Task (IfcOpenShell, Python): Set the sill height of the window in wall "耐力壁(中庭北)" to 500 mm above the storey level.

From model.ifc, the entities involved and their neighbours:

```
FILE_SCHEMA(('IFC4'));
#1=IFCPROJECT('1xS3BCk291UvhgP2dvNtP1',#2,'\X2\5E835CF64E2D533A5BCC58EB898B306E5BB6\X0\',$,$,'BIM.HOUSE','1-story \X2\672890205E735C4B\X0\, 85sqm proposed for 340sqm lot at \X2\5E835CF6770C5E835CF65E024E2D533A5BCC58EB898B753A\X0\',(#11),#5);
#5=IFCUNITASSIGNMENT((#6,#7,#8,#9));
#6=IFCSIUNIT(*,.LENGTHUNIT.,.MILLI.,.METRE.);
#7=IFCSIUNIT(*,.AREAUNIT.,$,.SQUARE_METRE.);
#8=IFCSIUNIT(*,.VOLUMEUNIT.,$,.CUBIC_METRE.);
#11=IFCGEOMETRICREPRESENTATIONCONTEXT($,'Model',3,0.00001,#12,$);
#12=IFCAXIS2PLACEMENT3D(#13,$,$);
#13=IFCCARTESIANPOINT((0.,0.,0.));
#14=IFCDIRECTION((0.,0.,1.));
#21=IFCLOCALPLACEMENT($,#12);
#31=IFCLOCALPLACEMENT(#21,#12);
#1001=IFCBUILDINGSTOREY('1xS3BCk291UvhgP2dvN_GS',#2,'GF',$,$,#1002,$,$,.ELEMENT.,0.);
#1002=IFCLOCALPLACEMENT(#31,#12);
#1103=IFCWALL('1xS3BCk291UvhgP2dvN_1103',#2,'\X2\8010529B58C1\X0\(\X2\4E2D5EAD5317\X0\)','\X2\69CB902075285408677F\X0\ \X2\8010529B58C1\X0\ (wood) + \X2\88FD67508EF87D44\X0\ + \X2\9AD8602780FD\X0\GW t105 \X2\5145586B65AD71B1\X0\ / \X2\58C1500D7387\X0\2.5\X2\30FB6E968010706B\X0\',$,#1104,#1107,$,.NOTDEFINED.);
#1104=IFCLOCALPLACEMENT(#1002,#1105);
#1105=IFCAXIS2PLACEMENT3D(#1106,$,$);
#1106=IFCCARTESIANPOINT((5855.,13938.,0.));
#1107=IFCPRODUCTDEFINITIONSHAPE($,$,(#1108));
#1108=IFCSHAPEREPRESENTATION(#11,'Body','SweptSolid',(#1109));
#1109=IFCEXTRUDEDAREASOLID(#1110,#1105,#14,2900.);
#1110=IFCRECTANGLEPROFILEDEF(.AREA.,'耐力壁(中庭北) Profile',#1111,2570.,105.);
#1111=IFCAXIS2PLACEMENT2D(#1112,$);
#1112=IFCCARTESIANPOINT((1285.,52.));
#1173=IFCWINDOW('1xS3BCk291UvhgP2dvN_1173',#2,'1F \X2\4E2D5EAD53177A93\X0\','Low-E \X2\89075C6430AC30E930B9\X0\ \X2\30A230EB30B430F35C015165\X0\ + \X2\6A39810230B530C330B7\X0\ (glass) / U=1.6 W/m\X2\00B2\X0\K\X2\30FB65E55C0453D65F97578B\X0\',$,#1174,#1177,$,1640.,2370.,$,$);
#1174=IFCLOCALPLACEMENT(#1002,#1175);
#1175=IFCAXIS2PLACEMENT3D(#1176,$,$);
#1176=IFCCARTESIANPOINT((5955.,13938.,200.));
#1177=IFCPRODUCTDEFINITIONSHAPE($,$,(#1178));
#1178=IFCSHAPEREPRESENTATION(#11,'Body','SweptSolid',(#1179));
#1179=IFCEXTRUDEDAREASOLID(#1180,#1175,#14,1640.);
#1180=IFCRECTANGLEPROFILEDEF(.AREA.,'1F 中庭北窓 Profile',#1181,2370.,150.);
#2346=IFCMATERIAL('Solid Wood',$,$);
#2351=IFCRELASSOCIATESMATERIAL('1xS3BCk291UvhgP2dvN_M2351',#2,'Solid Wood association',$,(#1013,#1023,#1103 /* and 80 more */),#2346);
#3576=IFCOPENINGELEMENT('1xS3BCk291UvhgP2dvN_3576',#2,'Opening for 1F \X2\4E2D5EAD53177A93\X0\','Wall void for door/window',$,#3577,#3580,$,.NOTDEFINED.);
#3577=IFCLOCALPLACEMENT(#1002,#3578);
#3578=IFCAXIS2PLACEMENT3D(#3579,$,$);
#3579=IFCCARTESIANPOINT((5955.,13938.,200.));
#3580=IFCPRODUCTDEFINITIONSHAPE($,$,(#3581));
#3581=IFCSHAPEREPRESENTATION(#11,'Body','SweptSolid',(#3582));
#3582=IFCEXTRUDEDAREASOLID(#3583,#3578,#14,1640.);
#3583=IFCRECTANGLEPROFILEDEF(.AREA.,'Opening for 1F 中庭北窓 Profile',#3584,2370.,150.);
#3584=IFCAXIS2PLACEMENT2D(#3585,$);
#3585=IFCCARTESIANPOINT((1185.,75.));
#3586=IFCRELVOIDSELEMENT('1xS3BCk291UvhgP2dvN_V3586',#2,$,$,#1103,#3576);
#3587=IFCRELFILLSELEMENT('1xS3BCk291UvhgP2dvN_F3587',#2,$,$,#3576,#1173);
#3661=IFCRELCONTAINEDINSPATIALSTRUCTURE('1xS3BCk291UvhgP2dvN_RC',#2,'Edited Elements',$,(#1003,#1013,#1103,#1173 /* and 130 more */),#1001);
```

```python
import numpy as np
import ifcopenshell
import ifcopenshell.api.geometry
import ifcopenshell.geom
import ifcopenshell.util.element
import ifcopenshell.util.placement
import ifcopenshell.util.shape
import ifcopenshell.util.unit

model = ifcopenshell.open("model.ifc")
unit_scale = ifcopenshell.util.unit.calculate_unit_scale(model)

window = model.by_guid("1xS3BCk291UvhgP2dvN_1173")
opening = window.FillsVoids[0].RelatingOpeningElement
storey = ifcopenshell.util.element.get_container(window, ifc_class="IfcBuildingStorey")
level = ifcopenshell.util.placement.get_local_placement(storey.ObjectPlacement)[2, 3]

# The opening's origin need not be at the sill, so measure its lowest point.
shape = ifcopenshell.geom.create_shape(ifcopenshell.geom.settings(), opening)
bottom = ifcopenshell.util.shape.get_shape_bottom_elevation(shape, shape.geometry) / unit_scale
dz = level + 500.0 - bottom

shift = np.array([0.0, 0.0, dz])
# The window is not placed relative to its opening, so move both.
for product in (opening, window):
    matrix = ifcopenshell.util.placement.get_local_placement(product.ObjectPlacement)
    matrix[:3, 3] += shift
    ifcopenshell.api.geometry.edit_object_placement(model, product=product, matrix=matrix, is_si=False)

print(f"moved by {dz * unit_scale:+.3f} m")

model.write("model_updated.ifc")
```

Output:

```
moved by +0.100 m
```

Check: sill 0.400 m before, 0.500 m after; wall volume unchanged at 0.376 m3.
